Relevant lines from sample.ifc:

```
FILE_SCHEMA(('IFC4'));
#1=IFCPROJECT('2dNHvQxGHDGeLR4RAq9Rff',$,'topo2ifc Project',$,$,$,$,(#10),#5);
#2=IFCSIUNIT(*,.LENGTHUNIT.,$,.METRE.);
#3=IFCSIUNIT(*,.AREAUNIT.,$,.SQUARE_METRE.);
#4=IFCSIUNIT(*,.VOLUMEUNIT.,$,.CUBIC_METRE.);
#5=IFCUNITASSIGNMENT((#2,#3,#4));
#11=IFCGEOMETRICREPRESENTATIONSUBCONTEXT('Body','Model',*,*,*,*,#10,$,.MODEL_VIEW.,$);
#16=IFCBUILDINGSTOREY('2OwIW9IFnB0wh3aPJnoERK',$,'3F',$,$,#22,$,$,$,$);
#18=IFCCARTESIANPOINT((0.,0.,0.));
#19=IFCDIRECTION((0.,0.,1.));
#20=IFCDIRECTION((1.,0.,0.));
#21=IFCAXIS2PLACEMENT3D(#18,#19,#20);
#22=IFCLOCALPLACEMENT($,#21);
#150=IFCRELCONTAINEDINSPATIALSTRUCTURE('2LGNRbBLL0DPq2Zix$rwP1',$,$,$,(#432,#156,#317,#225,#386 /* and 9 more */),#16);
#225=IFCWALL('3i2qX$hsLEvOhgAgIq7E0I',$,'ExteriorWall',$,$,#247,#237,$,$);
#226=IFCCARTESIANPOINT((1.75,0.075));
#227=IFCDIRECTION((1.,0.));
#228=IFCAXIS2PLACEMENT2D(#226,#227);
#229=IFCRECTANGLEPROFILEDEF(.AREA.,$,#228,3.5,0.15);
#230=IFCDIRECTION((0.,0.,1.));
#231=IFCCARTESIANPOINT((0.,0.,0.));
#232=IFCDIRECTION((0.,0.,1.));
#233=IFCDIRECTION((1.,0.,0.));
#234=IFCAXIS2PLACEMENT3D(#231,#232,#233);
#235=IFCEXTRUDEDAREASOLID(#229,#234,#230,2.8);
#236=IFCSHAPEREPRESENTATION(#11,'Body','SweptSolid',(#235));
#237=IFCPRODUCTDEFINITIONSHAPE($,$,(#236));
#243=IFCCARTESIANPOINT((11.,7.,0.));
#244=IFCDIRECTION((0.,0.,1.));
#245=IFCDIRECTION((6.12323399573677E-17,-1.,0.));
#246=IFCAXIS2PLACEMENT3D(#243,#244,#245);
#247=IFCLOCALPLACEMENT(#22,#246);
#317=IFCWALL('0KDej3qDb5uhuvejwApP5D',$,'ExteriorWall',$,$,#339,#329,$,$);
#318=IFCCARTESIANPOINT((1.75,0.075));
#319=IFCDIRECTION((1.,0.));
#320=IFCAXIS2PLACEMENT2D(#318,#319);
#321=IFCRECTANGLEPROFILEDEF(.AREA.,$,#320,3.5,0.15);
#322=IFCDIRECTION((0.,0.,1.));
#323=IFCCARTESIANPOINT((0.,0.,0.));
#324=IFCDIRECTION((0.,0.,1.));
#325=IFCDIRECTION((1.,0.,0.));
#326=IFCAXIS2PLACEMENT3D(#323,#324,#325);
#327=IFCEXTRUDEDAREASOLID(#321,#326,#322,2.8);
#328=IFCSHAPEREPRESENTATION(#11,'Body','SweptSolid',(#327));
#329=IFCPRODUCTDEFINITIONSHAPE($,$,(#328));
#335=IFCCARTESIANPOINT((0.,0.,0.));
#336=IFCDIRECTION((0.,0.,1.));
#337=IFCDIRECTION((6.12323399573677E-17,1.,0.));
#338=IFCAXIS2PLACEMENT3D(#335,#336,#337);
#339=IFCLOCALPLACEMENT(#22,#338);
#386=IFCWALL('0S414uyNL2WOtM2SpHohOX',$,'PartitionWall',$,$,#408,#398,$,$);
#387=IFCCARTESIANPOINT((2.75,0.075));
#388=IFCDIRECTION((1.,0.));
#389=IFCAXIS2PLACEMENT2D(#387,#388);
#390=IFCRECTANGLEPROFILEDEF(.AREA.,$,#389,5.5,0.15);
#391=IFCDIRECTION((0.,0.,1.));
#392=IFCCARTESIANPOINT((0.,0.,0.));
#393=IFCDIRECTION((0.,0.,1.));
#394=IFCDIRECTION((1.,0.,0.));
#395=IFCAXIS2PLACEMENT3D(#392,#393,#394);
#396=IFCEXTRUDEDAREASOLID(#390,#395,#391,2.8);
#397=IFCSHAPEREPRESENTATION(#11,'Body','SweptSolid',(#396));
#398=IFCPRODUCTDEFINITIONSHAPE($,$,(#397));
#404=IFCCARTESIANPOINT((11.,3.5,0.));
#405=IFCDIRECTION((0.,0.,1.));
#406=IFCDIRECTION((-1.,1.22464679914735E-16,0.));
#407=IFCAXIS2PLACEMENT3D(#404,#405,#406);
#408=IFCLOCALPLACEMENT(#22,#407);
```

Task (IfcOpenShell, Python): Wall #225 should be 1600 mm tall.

```python
import ifcopenshell
import ifcopenshell.geom
import ifcopenshell.util.representation
import ifcopenshell.util.shape
import ifcopenshell.util.unit

model = ifcopenshell.open("sample.ifc")
unit_scale = ifcopenshell.util.unit.calculate_unit_scale(model)
settings = ifcopenshell.geom.settings()


def volume(element):
    """Net volume in cubic metres, openings subtracted."""
    shape = ifcopenshell.geom.create_shape(settings, element)
    return ifcopenshell.util.shape.get_volume(shape.geometry)


wall = model.by_id(225)
before = volume(wall)

body = ifcopenshell.util.representation.get_representation(wall, "Model", "Body")
solid = body.Items[0]
old_height = solid.Depth
solid.Depth = 1.6 / unit_scale
after = volume(wall)

print(f"height {old_height:g} -> {solid.Depth:g}, volume {before:.3f} -> {after:.3f} m3")

model.write("sample_v2.ifc")
```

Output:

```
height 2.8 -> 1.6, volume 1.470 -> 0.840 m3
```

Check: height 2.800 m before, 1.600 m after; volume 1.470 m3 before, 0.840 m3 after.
